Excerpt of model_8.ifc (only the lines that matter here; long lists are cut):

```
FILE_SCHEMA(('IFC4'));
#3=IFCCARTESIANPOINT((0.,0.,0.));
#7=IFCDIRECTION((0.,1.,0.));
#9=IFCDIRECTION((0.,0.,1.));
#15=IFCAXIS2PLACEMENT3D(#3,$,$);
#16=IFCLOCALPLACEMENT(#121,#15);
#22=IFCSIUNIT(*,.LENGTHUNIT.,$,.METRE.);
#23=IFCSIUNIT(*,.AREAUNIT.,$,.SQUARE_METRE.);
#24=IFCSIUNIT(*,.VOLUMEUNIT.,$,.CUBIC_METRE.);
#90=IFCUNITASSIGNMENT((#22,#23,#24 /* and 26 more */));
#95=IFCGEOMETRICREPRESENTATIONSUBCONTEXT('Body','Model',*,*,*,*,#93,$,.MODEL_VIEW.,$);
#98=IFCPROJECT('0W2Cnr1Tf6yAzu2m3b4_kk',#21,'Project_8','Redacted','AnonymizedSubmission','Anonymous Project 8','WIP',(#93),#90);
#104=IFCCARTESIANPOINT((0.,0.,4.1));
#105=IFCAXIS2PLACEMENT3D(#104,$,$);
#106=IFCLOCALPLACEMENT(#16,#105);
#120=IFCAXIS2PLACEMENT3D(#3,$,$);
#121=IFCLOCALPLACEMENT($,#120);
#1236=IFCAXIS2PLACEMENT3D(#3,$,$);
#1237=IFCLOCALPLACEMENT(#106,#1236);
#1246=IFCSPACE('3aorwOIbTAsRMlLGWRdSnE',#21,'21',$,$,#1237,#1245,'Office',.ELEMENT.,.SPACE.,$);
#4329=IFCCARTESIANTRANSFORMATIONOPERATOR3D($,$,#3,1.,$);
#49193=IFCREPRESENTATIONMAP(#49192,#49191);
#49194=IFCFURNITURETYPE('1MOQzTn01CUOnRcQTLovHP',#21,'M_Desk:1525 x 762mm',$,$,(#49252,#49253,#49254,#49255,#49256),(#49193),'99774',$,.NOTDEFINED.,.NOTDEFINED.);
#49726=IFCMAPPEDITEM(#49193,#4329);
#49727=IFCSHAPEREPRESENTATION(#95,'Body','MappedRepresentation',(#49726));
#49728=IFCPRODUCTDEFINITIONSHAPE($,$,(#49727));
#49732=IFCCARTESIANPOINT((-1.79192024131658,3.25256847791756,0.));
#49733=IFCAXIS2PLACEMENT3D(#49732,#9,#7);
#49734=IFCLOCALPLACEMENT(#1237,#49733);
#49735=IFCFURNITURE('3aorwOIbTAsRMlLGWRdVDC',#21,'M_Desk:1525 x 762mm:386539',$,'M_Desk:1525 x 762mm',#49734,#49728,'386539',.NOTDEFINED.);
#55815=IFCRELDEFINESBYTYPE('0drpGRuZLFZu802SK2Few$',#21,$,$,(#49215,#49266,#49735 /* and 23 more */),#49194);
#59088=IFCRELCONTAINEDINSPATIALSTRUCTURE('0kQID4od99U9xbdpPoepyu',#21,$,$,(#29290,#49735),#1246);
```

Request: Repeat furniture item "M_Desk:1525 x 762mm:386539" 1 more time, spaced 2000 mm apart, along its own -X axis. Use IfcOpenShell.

```python
import ifcopenshell
import ifcopenshell.api.geometry
import ifcopenshell.api.root
import ifcopenshell.util.element
import ifcopenshell.util.placement

model = ifcopenshell.open("model_8.ifc")


def reuse_history(source, copy):
    """copy_class also copies each property set's owner history, people and application; keep the originals."""
    for rel in copy.IsDefinedBy:
        if rel.is_a("IfcRelDefinesByProperties") and (history := rel.RelatingPropertyDefinition.OwnerHistory):
            rel.RelatingPropertyDefinition.OwnerHistory = source.OwnerHistory
            ifcopenshell.util.element.remove_deep2(model, history)


source = model.by_guid("3aorwOIbTAsRMlLGWRdVDC")
base = ifcopenshell.util.placement.get_local_placement(source.ObjectPlacement)
step = -base[:3, 0] * 2.0

for i in range(1, 2):
    copy = ifcopenshell.api.root.copy_class(model, product=source)
    copy.Representation = ifcopenshell.util.element.copy_deep(
        model, source.Representation, exclude=["IfcGeometricRepresentationContext", "IfcRepresentationMap"]
    )
    copy.Name = "M_Desk:1525 x 762mm"
    copy.Tag = None
    reuse_history(source, copy)
    matrix = base.copy()
    matrix[:3, 3] += i * step
    print("added at", matrix[:3, 3].round(3) + 0.0)
    ifcopenshell.api.geometry.edit_object_placement(model, product=copy, matrix=matrix, is_si=False)

model.write("model_8_v2.ifc")
```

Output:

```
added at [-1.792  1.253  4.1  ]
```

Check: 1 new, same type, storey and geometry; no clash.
